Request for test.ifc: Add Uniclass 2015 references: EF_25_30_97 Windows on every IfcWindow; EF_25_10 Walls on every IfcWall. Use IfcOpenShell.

First a look at what the model holds.

```python
import ifcopenshell

model = ifcopenshell.open("test.ifc")
print(model.schema)
print("classifications:", [c.Name for c in model.by_type("IfcClassification")])
for ifc_class in ("IfcDoor", "IfcRoof", "IfcStair", "IfcWall", "IfcWindow"):
    print(ifc_class, len(model.by_type(ifc_class)))
```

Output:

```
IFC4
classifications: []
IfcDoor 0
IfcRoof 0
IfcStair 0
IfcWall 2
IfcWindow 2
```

```python
import ifcopenshell
import ifcopenshell.api.classification

model = ifcopenshell.open("test.ifc")

system = ifcopenshell.api.classification.add_classification(model, classification="Uniclass 2015")

codes = {
    "IfcWindow": ("EF_25_30_97", "Windows"),
    "IfcWall": ("EF_25_10", "Walls"),
}
for ifc_class, (code, name) in codes.items():
    products = model.by_type(ifc_class)
    ifcopenshell.api.classification.add_reference(
        model, products=products, classification=system, identification=code, name=name
    )
    print(code, len(products))

model.write("test_v2.ifc")
```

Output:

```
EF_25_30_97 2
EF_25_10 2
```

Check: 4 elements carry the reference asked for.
